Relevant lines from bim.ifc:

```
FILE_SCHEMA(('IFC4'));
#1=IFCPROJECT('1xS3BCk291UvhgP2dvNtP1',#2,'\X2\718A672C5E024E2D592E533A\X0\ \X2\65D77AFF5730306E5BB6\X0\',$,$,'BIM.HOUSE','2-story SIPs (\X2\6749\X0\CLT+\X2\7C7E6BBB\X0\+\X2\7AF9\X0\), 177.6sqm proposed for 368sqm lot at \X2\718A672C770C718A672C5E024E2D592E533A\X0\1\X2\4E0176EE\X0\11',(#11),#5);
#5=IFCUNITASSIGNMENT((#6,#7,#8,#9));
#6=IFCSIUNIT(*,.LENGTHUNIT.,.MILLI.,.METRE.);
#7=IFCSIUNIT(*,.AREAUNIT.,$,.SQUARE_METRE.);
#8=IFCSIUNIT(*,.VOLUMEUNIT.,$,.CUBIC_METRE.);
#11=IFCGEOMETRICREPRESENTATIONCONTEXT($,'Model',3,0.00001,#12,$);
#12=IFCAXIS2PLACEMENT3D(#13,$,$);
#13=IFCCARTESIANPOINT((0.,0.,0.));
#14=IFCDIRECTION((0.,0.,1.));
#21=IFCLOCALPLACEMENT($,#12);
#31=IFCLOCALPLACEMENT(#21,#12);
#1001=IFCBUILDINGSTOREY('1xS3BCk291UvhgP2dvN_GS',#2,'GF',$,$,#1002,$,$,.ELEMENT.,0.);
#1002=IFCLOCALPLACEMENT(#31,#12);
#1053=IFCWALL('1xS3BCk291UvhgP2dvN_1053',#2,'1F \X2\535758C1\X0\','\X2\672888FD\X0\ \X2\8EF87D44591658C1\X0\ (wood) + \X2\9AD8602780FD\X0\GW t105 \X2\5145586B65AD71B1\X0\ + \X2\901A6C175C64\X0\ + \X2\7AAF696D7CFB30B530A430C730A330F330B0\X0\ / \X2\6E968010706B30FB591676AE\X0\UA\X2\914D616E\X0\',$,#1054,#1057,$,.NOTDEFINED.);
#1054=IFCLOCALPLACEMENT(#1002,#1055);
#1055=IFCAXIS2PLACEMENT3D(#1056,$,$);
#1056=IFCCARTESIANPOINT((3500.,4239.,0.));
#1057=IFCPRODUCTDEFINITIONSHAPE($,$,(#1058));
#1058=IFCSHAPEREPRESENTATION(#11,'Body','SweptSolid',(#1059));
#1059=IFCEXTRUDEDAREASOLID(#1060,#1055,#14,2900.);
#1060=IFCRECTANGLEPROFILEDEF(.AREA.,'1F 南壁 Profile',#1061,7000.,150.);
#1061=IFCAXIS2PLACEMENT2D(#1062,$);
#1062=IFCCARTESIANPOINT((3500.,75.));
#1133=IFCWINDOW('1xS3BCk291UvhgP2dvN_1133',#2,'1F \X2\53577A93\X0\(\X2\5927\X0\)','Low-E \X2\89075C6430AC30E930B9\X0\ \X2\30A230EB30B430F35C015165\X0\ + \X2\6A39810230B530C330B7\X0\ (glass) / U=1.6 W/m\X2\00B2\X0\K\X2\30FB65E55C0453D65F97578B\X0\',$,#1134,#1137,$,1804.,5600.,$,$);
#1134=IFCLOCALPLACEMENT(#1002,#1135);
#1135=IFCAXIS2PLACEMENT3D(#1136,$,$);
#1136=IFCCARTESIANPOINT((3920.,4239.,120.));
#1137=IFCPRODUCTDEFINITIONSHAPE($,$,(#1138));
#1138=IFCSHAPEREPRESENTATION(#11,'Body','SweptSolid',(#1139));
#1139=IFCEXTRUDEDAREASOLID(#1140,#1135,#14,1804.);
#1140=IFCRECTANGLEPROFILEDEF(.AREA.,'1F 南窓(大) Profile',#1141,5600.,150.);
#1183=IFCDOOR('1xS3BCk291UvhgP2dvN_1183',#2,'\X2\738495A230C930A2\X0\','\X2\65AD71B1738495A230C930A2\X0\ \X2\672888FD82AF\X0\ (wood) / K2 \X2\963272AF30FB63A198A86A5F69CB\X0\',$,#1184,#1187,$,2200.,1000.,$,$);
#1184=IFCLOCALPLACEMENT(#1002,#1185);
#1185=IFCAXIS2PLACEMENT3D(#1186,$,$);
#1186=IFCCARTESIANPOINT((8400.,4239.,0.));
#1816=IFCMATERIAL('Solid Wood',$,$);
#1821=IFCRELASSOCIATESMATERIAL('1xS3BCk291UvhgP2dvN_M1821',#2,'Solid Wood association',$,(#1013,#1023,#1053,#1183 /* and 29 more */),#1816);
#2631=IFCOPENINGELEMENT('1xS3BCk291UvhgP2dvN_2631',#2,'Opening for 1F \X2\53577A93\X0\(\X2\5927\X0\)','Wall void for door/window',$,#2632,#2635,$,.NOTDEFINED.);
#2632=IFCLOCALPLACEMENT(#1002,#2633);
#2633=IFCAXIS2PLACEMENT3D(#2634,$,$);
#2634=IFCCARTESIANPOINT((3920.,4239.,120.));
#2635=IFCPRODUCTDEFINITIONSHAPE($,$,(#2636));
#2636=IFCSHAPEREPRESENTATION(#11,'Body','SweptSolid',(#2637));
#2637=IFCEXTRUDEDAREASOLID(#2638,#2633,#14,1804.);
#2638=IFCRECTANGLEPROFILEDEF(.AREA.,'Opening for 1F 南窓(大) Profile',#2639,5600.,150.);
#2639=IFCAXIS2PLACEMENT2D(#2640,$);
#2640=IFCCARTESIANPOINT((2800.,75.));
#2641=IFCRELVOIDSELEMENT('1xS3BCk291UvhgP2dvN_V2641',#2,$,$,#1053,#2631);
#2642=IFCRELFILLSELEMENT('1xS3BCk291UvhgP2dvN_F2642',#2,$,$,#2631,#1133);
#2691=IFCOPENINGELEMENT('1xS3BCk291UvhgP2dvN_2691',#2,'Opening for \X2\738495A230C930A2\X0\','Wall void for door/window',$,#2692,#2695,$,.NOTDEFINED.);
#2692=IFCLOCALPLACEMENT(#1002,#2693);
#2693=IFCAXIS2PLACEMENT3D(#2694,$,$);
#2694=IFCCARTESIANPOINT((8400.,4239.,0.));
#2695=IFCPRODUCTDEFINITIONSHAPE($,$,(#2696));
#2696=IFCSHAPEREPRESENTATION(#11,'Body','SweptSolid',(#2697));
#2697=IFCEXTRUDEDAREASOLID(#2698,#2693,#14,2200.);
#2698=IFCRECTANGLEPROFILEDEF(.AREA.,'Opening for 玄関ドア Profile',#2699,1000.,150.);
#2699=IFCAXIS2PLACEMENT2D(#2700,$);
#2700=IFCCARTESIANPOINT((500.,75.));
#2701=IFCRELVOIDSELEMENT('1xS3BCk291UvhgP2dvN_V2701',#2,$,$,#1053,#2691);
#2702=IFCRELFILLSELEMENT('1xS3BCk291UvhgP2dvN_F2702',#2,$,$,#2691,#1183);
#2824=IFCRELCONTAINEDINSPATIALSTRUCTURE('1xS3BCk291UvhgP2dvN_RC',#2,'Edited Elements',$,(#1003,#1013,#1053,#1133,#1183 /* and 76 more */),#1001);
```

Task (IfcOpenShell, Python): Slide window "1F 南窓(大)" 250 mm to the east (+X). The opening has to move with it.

```python
import ifcopenshell
import ifcopenshell.api.geometry
import ifcopenshell.util.placement

model = ifcopenshell.open("bim.ifc")

window = model.by_guid("1xS3BCk291UvhgP2dvN_1133")
opening = window.FillsVoids[0].RelatingOpeningElement
wall = opening.VoidsElements[0].RelatingBuildingElement

wall_matrix = ifcopenshell.util.placement.get_local_placement(wall.ObjectPlacement)
shift = wall_matrix[:3, 0] * 250.0
before = ifcopenshell.util.placement.get_local_placement(window.ObjectPlacement)[:3, 3].copy()

# The window is not placed relative to its opening, so move both.
for product in (opening, window):
    matrix = ifcopenshell.util.placement.get_local_placement(product.ObjectPlacement)
    matrix[:3, 3] += shift
    ifcopenshell.api.geometry.edit_object_placement(model, product=product, matrix=matrix, is_si=False)

after = ifcopenshell.util.placement.get_local_placement(window.ObjectPlacement)[:3, 3]
print("window moved by", (after - before).round(3) + 0.0)

model.write("bim_edited.ifc")
```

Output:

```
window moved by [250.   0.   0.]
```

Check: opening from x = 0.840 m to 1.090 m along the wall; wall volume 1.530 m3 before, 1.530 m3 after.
